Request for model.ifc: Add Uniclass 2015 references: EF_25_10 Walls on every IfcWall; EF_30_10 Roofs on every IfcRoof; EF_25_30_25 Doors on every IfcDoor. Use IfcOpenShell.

First a look at what the model holds.

```python
import ifcopenshell

model = ifcopenshell.open("model.ifc")
print(model.schema)
print("classifications:", [c.Name for c in model.by_type("IfcClassification")])
for ifc_class in ("IfcDoor", "IfcRoof", "IfcStair", "IfcWall", "IfcWindow"):
    print(ifc_class, len(model.by_type(ifc_class)))
```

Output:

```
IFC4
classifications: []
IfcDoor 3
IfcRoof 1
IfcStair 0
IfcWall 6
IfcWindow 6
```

```python
import ifcopenshell
import ifcopenshell.api.classification

model = ifcopenshell.open("model.ifc")

system = ifcopenshell.api.classification.add_classification(model, classification="Uniclass 2015")

codes = {
    "IfcWall": ("EF_25_10", "Walls"),
    "IfcRoof": ("EF_30_10", "Roofs"),
    "IfcDoor": ("EF_25_30_25", "Doors"),
}
for ifc_class, (code, name) in codes.items():
    products = model.by_type(ifc_class)
    ifcopenshell.api.classification.add_reference(
        model, products=products, classification=system, identification=code, name=name
    )
    print(code, len(products))

model.write("model_rev.ifc")
```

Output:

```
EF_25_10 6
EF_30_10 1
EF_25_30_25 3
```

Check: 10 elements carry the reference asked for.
